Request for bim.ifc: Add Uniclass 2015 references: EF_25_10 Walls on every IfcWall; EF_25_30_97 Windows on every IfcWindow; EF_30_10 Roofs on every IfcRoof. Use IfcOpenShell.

First a look at what the model holds.

```python
import ifcopenshell

model = ifcopenshell.open("bim.ifc")
print(model.schema)
print("classifications:", [c.Name for c in model.by_type("IfcClassification")])
for ifc_class in ("IfcDoor", "IfcRoof", "IfcStair", "IfcWall", "IfcWindow"):
    print(ifc_class, len(model.by_type(ifc_class)))
```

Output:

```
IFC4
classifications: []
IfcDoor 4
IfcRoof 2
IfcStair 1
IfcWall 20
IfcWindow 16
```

```python
import ifcopenshell
import ifcopenshell.api.classification

model = ifcopenshell.open("bim.ifc")

system = ifcopenshell.api.classification.add_classification(model, classification="Uniclass 2015")

codes = {
    "IfcWall": ("EF_25_10", "Walls"),
    "IfcWindow": ("EF_25_30_97", "Windows"),
    "IfcRoof": ("EF_30_10", "Roofs"),
}
for ifc_class, (code, name) in codes.items():
    products = model.by_type(ifc_class)
    ifcopenshell.api.classification.add_reference(
        model, products=products, classification=system, identification=code, name=name
    )
    print(code, len(products))

model.write("bim-out.ifc")
```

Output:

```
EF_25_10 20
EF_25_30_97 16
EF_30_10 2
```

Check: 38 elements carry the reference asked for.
